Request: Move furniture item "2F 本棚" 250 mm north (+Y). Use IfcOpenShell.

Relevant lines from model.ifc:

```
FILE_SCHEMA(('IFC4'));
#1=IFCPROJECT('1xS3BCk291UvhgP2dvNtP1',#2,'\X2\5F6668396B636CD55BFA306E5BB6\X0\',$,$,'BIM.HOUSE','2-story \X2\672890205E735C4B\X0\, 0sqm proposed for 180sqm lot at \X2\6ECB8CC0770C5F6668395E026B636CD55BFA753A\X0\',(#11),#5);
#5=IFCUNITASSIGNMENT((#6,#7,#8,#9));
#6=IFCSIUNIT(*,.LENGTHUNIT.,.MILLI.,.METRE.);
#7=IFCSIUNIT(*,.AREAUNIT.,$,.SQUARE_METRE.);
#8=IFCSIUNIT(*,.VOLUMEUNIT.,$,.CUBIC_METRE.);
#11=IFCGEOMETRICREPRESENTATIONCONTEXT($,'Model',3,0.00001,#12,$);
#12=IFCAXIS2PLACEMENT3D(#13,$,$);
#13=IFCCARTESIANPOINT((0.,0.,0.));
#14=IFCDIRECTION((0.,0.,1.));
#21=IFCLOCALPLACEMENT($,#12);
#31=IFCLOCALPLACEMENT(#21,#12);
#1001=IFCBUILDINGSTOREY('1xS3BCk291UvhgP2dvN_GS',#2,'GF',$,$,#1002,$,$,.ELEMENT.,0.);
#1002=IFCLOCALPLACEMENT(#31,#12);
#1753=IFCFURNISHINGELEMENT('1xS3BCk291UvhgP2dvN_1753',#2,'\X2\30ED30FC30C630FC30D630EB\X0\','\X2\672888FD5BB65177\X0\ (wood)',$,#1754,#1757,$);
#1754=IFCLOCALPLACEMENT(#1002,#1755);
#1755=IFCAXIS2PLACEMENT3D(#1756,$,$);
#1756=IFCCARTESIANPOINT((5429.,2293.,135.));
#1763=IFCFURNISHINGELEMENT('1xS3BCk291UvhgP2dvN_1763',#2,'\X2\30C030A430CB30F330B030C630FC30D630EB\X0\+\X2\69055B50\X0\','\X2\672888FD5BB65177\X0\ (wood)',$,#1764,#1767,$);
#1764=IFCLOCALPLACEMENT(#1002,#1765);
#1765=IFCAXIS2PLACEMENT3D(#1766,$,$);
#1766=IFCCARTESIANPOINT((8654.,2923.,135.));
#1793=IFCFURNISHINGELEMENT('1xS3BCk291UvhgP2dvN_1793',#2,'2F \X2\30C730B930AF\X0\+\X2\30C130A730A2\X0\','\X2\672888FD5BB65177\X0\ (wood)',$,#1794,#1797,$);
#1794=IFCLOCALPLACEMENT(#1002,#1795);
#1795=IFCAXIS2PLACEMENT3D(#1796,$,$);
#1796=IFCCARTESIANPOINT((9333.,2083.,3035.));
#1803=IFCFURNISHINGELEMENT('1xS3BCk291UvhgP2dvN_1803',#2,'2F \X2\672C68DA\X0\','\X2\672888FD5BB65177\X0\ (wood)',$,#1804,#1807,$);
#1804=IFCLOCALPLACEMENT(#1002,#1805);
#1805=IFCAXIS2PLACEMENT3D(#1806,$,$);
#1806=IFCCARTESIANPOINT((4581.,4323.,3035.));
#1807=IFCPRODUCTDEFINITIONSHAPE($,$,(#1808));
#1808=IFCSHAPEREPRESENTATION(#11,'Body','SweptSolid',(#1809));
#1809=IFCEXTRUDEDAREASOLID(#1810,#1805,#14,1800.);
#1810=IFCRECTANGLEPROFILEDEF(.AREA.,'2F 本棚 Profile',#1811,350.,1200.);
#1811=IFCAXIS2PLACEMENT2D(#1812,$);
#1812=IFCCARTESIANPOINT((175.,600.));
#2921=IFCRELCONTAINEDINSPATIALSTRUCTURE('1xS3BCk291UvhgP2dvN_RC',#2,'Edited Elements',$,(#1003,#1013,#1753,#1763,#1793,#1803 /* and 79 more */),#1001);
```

```python
import ifcopenshell
import ifcopenshell.api.geometry
import ifcopenshell.util.placement
import ifcopenshell.util.unit

model = ifcopenshell.open("model.ifc")
unit_scale = ifcopenshell.util.unit.calculate_unit_scale(model)

item = model.by_guid("1xS3BCk291UvhgP2dvN_1803")
matrix = ifcopenshell.util.placement.get_local_placement(item.ObjectPlacement)
matrix[1, 3] += 0.25 / unit_scale
ifcopenshell.api.geometry.edit_object_placement(model, product=item, matrix=matrix, is_si=False)

print(ifcopenshell.util.placement.get_local_placement(item.ObjectPlacement).round(3) + 0.0)

model.write("model_edited.ifc")
```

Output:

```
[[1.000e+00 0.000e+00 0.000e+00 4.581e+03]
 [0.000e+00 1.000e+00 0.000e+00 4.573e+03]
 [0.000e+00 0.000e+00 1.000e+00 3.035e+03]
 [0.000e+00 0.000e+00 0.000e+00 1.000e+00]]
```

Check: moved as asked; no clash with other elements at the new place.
